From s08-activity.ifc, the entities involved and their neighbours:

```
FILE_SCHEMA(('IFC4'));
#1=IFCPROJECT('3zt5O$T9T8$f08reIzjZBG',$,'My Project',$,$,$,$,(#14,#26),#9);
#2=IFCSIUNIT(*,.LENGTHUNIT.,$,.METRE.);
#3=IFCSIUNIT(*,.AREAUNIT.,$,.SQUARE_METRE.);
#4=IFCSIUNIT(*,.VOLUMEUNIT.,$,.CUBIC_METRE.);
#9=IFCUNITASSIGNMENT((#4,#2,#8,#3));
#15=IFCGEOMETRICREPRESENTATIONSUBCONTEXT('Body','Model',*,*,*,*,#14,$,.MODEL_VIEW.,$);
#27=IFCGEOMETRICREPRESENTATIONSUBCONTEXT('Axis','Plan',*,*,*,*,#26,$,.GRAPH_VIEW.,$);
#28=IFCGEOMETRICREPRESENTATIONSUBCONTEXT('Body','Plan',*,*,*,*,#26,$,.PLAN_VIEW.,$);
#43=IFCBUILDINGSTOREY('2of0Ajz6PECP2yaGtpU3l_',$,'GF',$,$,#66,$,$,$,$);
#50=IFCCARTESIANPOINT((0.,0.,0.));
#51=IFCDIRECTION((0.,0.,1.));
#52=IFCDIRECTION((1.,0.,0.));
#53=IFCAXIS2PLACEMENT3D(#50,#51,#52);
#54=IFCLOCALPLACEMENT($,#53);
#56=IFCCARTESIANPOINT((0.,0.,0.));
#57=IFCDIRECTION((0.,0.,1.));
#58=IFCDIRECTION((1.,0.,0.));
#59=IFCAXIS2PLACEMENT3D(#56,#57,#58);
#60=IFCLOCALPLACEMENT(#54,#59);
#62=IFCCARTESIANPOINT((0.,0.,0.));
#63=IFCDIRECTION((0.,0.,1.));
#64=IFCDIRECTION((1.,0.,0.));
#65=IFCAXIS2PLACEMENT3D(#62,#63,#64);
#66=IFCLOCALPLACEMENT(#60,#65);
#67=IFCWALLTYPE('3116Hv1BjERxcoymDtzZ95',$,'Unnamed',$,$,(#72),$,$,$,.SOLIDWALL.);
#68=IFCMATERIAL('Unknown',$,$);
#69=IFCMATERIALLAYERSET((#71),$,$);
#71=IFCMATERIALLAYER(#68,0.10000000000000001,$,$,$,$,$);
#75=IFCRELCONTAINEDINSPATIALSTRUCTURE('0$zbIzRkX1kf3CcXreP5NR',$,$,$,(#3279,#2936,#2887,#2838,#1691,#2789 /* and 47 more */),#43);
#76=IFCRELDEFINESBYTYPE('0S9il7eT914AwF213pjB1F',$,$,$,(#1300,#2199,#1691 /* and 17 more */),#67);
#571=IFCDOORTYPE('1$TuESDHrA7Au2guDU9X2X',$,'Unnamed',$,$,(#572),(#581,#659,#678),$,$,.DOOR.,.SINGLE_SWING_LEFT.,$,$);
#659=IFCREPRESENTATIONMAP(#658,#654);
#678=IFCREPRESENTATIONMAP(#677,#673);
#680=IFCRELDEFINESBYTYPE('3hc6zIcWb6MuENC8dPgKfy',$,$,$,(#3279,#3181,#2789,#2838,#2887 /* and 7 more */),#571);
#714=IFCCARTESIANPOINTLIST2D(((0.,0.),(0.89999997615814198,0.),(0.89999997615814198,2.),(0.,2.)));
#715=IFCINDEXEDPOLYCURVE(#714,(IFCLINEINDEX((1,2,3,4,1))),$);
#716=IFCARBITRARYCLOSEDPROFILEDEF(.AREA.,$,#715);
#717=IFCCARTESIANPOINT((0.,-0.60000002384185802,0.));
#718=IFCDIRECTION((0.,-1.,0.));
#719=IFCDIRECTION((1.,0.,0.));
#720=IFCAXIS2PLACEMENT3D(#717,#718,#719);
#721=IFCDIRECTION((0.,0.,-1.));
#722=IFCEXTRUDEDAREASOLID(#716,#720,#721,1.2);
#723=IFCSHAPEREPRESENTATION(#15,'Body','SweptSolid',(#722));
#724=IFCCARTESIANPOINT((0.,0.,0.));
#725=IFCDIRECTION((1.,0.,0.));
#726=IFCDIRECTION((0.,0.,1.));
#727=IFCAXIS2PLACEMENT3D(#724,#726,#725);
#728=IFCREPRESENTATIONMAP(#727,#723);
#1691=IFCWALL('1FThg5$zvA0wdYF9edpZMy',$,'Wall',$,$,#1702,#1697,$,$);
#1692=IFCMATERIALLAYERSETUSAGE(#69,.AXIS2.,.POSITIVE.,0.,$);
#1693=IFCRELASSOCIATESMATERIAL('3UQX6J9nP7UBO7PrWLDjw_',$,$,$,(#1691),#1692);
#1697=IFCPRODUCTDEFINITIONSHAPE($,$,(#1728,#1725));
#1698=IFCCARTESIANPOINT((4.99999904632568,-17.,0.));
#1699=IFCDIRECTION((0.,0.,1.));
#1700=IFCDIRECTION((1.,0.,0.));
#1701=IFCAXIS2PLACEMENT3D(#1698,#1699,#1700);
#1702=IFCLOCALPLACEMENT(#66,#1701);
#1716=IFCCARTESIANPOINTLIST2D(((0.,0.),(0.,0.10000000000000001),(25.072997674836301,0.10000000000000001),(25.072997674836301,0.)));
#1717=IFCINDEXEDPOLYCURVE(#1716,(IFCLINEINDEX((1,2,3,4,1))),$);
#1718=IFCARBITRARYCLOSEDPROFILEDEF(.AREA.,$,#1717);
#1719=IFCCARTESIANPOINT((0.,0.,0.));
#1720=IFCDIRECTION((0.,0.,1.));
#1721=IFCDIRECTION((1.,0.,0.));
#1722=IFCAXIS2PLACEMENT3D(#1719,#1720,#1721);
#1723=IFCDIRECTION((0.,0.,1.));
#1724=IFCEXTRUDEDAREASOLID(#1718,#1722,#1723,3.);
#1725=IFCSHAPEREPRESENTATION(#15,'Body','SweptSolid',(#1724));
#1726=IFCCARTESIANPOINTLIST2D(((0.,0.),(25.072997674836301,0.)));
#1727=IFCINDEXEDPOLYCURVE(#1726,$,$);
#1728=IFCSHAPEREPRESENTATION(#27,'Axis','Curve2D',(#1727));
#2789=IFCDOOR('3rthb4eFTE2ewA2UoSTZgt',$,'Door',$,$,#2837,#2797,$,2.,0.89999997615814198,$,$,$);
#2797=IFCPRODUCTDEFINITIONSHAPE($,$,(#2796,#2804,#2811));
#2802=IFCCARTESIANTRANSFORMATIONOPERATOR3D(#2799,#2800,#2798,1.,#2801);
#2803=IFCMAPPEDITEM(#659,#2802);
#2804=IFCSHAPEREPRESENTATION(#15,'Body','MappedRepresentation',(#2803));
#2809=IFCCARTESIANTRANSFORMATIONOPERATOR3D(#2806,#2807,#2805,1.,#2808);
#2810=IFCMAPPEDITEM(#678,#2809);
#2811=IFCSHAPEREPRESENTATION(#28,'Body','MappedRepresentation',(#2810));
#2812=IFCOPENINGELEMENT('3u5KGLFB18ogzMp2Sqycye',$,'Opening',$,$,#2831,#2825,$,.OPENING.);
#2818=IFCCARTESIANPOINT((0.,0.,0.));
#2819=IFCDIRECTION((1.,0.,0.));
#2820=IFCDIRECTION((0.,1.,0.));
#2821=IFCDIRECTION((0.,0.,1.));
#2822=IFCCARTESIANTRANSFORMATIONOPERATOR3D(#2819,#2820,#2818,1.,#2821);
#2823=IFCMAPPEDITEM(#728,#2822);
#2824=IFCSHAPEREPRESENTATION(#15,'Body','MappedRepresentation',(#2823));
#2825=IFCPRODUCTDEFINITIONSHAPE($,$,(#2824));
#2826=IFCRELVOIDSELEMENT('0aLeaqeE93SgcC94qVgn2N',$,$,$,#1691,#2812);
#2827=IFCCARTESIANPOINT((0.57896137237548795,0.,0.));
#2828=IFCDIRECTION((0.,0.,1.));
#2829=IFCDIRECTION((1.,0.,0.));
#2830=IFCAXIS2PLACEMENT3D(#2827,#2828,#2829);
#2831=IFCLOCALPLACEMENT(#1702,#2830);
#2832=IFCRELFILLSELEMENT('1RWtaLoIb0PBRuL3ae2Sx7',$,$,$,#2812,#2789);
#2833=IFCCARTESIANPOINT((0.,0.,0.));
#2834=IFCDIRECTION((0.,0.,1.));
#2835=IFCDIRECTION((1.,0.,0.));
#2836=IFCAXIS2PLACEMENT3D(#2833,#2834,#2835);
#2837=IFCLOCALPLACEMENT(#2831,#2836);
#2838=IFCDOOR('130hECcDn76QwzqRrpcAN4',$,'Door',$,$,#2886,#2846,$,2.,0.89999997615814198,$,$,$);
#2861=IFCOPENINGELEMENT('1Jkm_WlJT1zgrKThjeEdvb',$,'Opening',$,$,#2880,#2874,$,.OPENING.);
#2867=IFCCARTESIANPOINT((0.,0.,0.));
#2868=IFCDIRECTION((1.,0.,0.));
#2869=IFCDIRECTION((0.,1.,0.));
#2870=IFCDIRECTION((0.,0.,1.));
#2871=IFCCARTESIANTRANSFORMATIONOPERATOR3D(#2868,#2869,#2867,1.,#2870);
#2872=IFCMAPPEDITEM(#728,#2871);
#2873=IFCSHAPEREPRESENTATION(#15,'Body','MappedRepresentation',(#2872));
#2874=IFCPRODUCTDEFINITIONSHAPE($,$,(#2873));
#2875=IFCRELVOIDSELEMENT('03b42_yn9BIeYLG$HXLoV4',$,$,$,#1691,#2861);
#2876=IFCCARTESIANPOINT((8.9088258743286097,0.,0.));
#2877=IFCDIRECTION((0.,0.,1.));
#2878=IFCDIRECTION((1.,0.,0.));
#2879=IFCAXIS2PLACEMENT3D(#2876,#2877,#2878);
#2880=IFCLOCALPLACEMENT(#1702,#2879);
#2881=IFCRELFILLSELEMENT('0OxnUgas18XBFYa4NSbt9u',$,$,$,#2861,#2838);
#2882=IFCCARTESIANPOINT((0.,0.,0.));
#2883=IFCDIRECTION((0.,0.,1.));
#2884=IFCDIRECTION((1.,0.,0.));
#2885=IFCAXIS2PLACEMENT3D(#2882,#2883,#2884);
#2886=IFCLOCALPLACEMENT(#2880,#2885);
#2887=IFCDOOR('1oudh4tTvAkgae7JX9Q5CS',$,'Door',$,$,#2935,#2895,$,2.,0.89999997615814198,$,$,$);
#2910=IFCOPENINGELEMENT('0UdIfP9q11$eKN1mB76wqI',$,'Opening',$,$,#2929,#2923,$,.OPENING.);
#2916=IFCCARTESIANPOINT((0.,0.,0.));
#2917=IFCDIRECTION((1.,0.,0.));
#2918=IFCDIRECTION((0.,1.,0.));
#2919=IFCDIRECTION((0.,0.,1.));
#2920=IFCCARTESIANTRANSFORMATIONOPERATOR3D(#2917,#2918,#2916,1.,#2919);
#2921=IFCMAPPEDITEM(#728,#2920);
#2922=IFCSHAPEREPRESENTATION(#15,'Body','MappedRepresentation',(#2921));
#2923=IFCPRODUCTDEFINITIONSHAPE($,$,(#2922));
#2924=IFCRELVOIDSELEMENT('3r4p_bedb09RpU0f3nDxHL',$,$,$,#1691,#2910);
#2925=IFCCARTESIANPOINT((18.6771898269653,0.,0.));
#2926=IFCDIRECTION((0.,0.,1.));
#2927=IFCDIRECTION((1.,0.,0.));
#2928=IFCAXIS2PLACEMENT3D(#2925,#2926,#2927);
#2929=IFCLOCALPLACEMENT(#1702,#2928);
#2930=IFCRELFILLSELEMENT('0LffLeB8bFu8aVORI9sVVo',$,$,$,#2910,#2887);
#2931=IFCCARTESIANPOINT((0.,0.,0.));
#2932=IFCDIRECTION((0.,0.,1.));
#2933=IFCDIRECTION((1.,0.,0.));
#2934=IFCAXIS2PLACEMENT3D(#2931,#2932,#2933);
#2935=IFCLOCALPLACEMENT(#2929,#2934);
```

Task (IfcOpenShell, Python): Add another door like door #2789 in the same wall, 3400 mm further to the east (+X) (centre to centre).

```python
import ifcopenshell
import ifcopenshell.api.feature
import ifcopenshell.api.geometry
import ifcopenshell.api.root
import ifcopenshell.geom
import ifcopenshell.util.element
import ifcopenshell.util.placement
import ifcopenshell.util.shape

model = ifcopenshell.open("s08-activity.ifc")
settings = ifcopenshell.geom.settings()


def volume(element):
    """Net volume in cubic metres, openings subtracted."""
    shape = ifcopenshell.geom.create_shape(settings, element)
    return ifcopenshell.util.shape.get_volume(shape.geometry)


door = model.by_guid("3rthb4eFTE2ewA2UoSTZgt")
opening = door.FillsVoids[0].RelatingOpeningElement
wall = opening.VoidsElements[0].RelatingBuildingElement
before = volume(wall)
shift = ifcopenshell.util.placement.get_local_placement(wall.ObjectPlacement)[:3, 0] * 3.4

# copy_class copies the void relationship, type, container and properties, but no geometry.
new_opening = ifcopenshell.api.root.copy_class(model, product=opening)
new_opening.Representation = ifcopenshell.util.element.copy_deep(
    model, opening.Representation, exclude=["IfcGeometricRepresentationContext", "IfcRepresentationMap"]
)
new_door = ifcopenshell.api.root.copy_class(model, product=door)
new_door.Representation = ifcopenshell.util.element.copy_deep(
    model, door.Representation, exclude=["IfcGeometricRepresentationContext", "IfcRepresentationMap"]
)
ifcopenshell.api.feature.add_filling(model, opening=new_opening, element=new_door)

for old, new in ((opening, new_opening), (door, new_door)):
    matrix = ifcopenshell.util.placement.get_local_placement(old.ObjectPlacement)
    matrix[:3, 3] += shift
    ifcopenshell.api.geometry.edit_object_placement(model, product=new, matrix=matrix, is_si=False)

after = volume(wall)

print(f"wall volume {before:.3f} -> {after:.3f} m3")

model.write("s08-activity_rev.ifc")
```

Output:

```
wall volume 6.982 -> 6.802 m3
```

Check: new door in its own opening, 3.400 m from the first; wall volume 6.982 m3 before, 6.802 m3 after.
